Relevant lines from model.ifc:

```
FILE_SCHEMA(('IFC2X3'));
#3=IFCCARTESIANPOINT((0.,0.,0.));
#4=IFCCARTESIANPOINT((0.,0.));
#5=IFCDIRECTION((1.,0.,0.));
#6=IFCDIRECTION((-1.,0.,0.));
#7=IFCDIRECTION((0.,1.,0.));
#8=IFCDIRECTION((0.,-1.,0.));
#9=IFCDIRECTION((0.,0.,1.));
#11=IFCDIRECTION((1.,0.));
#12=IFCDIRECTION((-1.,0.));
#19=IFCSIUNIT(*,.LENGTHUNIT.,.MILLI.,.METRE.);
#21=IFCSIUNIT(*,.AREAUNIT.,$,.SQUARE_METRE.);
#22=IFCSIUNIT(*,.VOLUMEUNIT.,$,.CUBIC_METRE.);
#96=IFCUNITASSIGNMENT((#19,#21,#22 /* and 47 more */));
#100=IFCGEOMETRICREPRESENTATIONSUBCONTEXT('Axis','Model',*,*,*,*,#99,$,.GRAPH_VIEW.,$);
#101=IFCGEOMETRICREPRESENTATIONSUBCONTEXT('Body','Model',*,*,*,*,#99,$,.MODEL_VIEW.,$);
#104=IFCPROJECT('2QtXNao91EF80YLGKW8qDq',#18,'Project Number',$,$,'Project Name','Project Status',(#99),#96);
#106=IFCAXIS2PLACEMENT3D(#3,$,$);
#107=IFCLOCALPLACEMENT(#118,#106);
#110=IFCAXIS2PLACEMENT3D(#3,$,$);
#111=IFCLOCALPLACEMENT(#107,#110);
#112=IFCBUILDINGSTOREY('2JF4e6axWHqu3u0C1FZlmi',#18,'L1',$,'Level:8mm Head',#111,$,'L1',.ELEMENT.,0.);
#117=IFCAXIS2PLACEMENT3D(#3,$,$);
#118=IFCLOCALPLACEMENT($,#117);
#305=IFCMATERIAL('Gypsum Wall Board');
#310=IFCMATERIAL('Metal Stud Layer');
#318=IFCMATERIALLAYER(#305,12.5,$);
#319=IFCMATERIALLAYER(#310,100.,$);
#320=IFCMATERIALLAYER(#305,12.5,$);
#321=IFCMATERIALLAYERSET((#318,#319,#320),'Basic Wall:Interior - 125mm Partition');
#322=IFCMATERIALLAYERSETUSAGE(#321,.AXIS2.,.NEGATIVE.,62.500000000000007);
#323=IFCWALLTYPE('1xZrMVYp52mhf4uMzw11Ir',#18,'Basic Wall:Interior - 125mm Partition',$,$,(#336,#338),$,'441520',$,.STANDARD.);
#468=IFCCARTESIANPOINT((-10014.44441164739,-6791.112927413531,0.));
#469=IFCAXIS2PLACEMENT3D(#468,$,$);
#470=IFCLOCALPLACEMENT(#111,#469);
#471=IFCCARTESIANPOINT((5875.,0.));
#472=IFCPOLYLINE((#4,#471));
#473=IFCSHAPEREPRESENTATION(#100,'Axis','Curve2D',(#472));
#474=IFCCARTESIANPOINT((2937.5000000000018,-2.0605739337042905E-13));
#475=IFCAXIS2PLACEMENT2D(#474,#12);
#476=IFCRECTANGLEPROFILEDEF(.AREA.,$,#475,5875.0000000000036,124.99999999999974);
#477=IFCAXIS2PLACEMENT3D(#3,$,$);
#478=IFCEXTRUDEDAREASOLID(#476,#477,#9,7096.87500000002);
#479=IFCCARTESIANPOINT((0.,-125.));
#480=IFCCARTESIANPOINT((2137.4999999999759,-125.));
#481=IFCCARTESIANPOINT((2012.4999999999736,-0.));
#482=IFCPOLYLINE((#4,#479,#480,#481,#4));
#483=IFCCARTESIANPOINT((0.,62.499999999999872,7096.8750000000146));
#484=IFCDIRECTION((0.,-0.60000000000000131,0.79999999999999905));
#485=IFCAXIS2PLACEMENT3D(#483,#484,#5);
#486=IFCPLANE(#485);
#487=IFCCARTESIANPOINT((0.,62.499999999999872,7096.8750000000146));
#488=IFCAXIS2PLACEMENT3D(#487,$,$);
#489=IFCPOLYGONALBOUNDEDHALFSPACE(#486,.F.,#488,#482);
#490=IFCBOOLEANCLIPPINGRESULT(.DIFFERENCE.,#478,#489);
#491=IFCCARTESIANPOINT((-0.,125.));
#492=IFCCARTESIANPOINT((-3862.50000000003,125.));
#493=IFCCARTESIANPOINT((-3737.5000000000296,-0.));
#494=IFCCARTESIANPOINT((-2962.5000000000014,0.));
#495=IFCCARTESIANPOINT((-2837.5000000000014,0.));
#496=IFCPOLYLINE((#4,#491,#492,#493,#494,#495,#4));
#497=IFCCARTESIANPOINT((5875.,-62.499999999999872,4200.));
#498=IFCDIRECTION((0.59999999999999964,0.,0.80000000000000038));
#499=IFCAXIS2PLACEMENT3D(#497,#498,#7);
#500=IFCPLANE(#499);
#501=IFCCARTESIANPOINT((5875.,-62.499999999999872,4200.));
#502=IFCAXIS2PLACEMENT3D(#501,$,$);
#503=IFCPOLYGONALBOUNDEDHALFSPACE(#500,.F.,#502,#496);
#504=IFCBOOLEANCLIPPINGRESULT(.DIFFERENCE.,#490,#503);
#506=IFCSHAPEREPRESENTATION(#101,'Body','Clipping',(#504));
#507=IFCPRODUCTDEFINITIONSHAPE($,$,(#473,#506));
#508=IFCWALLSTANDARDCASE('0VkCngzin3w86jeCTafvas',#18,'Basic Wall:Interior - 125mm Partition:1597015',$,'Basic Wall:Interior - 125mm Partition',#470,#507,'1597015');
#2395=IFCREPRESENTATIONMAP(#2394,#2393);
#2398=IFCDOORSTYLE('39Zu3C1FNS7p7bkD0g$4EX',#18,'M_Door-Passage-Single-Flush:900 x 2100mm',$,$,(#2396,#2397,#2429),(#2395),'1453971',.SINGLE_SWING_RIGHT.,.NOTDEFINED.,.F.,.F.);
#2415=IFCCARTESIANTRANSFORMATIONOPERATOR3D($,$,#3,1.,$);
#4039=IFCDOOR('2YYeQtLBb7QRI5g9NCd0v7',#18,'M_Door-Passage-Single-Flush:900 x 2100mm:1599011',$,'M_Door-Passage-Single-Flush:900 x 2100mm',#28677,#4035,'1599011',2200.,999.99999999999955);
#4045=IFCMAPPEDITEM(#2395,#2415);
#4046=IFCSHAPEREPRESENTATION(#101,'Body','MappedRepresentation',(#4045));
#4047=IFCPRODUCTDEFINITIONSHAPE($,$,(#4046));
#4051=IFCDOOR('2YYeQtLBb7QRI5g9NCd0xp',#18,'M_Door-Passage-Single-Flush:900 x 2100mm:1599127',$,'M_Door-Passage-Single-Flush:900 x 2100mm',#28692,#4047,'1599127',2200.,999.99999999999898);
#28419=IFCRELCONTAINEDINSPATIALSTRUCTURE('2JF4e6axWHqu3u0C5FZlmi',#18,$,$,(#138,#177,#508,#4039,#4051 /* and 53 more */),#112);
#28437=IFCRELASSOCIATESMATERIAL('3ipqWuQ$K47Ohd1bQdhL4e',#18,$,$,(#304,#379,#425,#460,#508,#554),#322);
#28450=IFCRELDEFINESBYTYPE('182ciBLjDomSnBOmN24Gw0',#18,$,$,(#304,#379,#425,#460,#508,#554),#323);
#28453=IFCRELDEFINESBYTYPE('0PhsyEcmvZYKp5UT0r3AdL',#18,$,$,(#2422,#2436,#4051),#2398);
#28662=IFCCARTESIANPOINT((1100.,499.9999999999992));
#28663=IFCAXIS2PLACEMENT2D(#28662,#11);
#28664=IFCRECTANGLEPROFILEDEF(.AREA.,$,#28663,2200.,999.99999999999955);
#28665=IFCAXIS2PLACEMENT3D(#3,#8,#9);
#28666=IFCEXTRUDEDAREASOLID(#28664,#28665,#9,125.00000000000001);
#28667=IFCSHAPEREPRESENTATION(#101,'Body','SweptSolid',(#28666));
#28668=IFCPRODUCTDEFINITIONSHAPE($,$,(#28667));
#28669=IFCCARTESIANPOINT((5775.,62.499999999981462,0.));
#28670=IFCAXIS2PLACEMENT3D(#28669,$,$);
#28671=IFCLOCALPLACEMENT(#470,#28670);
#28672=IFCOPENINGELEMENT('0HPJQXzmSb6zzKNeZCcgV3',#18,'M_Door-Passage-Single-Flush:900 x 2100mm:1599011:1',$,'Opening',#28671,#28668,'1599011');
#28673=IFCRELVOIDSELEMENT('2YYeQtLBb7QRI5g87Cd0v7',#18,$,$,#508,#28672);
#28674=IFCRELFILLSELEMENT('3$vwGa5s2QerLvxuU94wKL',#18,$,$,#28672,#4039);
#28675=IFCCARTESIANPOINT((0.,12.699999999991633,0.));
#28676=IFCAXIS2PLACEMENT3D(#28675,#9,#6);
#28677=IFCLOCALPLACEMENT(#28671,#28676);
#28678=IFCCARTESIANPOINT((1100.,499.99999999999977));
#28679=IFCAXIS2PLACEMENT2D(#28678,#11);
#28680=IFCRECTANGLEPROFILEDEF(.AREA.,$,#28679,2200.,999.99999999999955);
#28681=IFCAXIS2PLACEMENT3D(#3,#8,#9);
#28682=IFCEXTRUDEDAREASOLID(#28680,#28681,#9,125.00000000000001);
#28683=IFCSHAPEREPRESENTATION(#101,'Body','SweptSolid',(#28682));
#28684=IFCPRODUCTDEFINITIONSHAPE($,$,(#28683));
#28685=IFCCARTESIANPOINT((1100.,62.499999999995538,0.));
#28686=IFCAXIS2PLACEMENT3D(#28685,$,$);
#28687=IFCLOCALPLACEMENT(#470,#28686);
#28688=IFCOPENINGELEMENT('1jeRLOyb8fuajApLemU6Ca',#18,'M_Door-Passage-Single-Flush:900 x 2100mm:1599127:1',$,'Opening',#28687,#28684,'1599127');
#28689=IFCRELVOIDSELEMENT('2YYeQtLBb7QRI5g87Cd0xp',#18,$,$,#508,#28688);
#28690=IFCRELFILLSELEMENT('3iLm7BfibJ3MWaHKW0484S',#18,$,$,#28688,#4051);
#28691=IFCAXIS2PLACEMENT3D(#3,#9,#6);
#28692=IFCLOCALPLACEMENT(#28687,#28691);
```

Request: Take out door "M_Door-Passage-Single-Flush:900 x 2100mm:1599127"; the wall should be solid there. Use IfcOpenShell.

```python
import ifcopenshell
import ifcopenshell.api.feature
import ifcopenshell.api.root
import ifcopenshell.geom
import ifcopenshell.util.shape

model = ifcopenshell.open("model.ifc")
settings = ifcopenshell.geom.settings()


def volume(element):
    """Net volume in cubic metres, openings subtracted."""
    shape = ifcopenshell.geom.create_shape(settings, element)
    return ifcopenshell.util.shape.get_volume(shape.geometry)


door = model.by_guid("2YYeQtLBb7QRI5g9NCd0xp")
opening = door.FillsVoids[0].RelatingOpeningElement
wall = opening.VoidsElements[0].RelatingBuildingElement
before = volume(wall)

ifcopenshell.api.root.remove_product(model, product=door)
ifcopenshell.api.feature.remove_feature(model, feature=opening)

after = volume(wall)

print(f"wall volume {before:.3f} -> {after:.3f} m3")

model.write("model-out.ifc")
```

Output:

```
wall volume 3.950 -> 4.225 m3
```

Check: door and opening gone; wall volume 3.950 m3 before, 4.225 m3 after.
